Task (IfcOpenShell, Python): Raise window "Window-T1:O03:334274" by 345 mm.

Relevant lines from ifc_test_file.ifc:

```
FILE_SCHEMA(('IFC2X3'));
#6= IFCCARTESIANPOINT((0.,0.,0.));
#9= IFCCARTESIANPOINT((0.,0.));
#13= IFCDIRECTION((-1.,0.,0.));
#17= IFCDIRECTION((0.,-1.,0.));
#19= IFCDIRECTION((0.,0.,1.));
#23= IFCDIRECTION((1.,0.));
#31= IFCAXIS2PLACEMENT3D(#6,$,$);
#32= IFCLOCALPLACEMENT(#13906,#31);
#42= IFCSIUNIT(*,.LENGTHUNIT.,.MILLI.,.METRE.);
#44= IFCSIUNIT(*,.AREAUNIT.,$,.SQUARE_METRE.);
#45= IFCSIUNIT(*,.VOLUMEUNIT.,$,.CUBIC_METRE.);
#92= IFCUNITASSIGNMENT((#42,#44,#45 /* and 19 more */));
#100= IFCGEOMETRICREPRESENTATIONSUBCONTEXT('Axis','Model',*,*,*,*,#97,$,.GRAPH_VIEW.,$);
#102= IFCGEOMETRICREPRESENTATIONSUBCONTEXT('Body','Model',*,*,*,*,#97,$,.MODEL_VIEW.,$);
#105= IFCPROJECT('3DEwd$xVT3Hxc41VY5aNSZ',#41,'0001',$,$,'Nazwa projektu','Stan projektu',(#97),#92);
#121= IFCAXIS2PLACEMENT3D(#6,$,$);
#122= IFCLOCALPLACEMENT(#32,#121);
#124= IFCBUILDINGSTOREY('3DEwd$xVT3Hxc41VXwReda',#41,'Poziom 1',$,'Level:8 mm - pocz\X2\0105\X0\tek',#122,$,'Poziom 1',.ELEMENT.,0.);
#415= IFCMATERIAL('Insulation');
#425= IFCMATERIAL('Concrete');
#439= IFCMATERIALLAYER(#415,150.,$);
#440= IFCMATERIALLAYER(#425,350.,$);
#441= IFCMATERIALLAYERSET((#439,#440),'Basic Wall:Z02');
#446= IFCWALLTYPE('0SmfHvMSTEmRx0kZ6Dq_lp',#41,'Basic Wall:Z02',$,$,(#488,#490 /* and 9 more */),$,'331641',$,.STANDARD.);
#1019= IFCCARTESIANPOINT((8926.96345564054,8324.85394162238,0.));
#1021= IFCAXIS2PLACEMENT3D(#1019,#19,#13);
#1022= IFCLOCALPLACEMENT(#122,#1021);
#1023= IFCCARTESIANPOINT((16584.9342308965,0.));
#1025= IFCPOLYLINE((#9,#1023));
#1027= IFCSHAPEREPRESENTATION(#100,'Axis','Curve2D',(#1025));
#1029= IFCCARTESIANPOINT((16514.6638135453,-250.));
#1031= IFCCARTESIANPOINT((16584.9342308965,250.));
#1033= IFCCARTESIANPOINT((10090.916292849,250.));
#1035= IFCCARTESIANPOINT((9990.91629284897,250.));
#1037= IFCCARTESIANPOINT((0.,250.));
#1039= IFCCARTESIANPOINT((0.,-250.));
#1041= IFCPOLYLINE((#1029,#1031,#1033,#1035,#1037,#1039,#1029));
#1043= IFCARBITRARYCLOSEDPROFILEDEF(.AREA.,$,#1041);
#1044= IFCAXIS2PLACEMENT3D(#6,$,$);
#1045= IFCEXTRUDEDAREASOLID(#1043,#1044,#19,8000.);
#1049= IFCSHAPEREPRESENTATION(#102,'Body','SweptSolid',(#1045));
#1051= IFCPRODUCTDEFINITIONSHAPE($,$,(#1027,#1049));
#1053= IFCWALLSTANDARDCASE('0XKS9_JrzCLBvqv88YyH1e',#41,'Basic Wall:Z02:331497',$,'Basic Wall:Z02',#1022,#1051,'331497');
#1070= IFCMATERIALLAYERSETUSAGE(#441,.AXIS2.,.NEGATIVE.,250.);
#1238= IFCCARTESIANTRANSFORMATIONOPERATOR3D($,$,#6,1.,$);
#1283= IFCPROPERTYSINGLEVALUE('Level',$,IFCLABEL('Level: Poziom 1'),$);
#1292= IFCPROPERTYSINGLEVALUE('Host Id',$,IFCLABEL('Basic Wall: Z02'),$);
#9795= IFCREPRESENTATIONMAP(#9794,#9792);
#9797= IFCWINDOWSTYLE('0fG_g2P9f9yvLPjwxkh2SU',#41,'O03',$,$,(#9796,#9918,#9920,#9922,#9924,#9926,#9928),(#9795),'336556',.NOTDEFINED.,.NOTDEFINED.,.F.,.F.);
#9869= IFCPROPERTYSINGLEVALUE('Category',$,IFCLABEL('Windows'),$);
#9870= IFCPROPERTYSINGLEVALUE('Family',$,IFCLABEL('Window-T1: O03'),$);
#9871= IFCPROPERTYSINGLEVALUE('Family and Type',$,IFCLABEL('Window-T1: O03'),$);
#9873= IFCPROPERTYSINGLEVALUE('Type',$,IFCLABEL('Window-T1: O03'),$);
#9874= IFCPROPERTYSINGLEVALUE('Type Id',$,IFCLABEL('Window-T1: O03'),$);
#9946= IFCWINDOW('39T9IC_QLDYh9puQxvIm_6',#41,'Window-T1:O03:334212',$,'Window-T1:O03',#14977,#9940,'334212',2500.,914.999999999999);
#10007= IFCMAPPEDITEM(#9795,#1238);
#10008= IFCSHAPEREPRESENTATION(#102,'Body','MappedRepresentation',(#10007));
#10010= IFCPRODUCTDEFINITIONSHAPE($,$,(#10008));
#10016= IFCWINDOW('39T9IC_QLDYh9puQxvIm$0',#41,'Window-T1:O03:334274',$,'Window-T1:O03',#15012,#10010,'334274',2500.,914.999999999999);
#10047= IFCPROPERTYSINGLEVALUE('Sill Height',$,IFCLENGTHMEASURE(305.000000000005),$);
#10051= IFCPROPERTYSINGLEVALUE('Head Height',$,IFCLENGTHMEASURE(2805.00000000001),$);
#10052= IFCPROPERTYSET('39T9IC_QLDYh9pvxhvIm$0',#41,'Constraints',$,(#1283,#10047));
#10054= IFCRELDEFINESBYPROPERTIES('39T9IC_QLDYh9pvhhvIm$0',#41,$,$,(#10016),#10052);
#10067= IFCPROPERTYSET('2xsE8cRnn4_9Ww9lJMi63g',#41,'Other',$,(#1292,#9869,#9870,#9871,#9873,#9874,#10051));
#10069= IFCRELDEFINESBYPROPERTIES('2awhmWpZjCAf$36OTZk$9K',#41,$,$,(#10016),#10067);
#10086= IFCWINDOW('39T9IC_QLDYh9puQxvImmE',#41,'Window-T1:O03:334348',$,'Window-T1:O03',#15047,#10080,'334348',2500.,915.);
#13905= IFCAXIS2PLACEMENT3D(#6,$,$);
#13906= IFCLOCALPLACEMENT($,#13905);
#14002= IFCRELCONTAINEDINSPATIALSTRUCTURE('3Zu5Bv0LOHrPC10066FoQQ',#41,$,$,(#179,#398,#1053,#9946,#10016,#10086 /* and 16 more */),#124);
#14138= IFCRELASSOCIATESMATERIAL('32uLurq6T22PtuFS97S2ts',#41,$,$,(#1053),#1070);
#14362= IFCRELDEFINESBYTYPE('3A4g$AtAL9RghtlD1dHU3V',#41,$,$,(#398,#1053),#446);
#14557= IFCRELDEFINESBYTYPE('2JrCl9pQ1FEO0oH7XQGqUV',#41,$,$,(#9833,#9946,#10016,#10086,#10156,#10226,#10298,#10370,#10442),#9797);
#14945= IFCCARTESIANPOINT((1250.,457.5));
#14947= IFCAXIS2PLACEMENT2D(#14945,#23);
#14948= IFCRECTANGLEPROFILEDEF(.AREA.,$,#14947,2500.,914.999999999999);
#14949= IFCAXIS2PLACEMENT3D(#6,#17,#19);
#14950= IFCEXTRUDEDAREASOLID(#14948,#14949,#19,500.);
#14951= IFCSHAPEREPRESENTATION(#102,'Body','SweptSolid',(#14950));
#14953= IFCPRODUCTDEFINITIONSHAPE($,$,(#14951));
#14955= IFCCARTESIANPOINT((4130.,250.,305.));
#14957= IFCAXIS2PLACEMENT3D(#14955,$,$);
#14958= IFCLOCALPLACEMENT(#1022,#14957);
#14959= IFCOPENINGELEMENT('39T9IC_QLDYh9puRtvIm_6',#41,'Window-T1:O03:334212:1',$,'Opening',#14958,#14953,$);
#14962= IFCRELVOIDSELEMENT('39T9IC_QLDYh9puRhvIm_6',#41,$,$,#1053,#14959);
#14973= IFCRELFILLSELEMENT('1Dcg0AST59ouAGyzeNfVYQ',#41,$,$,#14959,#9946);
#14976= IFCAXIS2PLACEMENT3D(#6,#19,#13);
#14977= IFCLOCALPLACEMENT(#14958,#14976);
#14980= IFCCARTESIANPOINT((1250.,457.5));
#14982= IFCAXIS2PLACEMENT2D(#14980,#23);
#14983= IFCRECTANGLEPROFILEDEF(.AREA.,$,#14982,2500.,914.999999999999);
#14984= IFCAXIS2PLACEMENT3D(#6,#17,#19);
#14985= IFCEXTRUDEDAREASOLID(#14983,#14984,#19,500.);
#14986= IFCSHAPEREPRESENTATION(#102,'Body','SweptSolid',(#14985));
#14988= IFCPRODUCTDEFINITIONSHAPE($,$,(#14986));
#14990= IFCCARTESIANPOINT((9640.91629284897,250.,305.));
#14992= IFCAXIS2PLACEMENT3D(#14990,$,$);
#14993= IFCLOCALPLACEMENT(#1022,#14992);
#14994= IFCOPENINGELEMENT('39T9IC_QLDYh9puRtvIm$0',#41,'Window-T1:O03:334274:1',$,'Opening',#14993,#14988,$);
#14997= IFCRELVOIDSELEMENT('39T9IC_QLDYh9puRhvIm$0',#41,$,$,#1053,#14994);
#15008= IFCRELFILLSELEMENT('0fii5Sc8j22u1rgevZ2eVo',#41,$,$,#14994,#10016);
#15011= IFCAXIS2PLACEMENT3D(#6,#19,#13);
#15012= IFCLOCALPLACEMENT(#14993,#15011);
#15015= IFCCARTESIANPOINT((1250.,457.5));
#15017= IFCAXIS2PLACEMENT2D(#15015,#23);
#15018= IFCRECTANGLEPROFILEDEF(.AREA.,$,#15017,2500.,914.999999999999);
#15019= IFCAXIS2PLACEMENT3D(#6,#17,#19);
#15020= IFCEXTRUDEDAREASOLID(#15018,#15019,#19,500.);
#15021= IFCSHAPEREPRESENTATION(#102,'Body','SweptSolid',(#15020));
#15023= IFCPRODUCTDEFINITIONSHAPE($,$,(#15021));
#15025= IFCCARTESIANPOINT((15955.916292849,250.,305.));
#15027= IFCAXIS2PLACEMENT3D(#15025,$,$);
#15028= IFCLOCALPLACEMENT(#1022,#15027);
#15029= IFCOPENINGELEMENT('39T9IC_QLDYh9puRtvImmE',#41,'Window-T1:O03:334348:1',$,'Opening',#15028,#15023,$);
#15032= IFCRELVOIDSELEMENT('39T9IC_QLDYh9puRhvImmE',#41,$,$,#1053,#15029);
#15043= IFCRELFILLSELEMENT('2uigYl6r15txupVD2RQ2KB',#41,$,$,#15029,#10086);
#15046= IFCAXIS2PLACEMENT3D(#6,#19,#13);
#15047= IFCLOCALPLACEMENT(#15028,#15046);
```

```python
import numpy as np
import ifcopenshell
import ifcopenshell.api.geometry
import ifcopenshell.api.pset
import ifcopenshell.util.element
import ifcopenshell.util.placement
import ifcopenshell.util.unit

model = ifcopenshell.open("ifc_test_file.ifc")
unit_scale = ifcopenshell.util.unit.calculate_unit_scale(model)

window = model.by_guid("39T9IC_QLDYh9puQxvIm$0")
opening = window.FillsVoids[0].RelatingOpeningElement
dz = 0.345 / unit_scale

shift = np.array([0.0, 0.0, dz])
# The window is placed relative to its opening, so it follows when the opening moves.
matrix = ifcopenshell.util.placement.get_local_placement(opening.ObjectPlacement)
matrix[:3, 3] += shift
ifcopenshell.api.geometry.edit_object_placement(
    model, product=opening, matrix=matrix, is_si=False, should_transform_children=True
)

# Keep the stored heights in step.
pset = model.by_id(ifcopenshell.util.element.get_pset(window, "Constraints", should_inherit=False)["id"])
ifcopenshell.api.pset.edit_pset(model, pset=pset, properties={
    "Sill Height": model.create_entity("IfcLengthMeasure", ifcopenshell.util.element.get_pset(window, "Constraints", "Sill Height") + dz),
})
pset = model.by_id(ifcopenshell.util.element.get_pset(window, "Other", should_inherit=False)["id"])
ifcopenshell.api.pset.edit_pset(model, pset=pset, properties={
    "Head Height": model.create_entity("IfcLengthMeasure", ifcopenshell.util.element.get_pset(window, "Other", "Head Height") + dz),
})

print(f"moved by {dz * unit_scale:+.3f} m")

model.write("ifc_test_file_v2.ifc")
```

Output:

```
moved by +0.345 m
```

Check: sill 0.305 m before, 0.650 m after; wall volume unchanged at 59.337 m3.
